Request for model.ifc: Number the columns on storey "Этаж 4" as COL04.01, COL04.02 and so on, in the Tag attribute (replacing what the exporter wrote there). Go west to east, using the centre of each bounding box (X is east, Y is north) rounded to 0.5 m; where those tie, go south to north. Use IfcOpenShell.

First a look at what the model holds.

```python
import ifcopenshell
import ifcopenshell.util.element
import ifcopenshell.util.placement

model = ifcopenshell.open("model.ifc")
print(model.schema)
storey = next(s for s in model.by_type("IfcBuildingStorey") if s.Name == "Этаж 4")
columns = [e for e in ifcopenshell.util.element.get_decomposition(storey) if e.is_a("IfcColumn")]
for e in sorted(columns, key=lambda e: e.id()):
    origin = ifcopenshell.util.placement.get_local_placement(e.ObjectPlacement)[:3, 3]
    print(e.id(), e.Tag, e.Name, origin.round(2) + 0.0, sep=" | ")
```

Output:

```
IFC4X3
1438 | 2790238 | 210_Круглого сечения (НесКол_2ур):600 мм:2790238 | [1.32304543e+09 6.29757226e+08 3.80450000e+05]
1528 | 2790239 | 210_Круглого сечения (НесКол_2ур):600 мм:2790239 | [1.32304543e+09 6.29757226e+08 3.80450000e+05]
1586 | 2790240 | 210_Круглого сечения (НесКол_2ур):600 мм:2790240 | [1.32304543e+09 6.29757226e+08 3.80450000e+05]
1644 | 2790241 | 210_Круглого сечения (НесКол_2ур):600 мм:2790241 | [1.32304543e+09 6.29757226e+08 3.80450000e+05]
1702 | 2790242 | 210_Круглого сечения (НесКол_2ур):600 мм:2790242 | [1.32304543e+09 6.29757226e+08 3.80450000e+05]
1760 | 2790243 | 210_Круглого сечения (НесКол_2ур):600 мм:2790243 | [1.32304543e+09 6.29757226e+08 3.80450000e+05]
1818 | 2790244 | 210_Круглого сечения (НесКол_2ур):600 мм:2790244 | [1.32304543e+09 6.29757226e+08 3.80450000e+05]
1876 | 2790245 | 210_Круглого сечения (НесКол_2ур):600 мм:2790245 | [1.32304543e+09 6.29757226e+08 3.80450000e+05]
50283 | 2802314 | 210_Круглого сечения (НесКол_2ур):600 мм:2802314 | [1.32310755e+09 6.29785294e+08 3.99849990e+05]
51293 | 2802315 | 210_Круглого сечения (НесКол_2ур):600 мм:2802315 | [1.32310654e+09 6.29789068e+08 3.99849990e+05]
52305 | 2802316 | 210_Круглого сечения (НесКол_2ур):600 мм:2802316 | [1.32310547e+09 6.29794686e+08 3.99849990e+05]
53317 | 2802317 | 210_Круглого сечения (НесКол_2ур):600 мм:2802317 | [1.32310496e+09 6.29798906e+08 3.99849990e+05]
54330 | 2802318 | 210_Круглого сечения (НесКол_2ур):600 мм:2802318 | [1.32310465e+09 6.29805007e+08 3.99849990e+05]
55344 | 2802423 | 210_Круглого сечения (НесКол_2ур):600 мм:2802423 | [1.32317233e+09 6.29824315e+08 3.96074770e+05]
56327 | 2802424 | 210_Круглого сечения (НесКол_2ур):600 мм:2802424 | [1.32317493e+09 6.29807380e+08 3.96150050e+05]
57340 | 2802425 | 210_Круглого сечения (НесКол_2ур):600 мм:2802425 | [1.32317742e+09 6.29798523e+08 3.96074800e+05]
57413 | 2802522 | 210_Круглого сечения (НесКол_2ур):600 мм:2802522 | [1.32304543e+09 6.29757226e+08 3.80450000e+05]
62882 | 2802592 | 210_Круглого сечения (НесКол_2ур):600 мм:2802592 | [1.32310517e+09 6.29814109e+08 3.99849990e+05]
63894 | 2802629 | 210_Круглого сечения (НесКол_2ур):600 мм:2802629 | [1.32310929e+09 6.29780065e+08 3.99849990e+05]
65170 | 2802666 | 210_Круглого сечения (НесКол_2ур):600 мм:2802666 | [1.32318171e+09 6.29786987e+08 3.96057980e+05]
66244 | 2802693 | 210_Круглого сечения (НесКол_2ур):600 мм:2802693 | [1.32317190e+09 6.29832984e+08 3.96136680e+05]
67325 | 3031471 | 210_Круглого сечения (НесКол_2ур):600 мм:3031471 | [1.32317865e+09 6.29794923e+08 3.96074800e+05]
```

```python
import ifcopenshell
import ifcopenshell.geom
import ifcopenshell.util.element
import ifcopenshell.util.shape

model = ifcopenshell.open("model.ifc")
settings = ifcopenshell.geom.settings()
settings.set("use-world-coords", True)


def centre(element):
    shape = ifcopenshell.geom.create_shape(settings, element)
    return ifcopenshell.util.shape.get_bbox_centroid(shape.geometry)


storey = next(s for s in model.by_type("IfcBuildingStorey") if s.Name == "Этаж 4")
columns = [e for e in ifcopenshell.util.element.get_decomposition(storey) if e.is_a("IfcColumn")]

# Insertion points can sit at a corner or the storey origin, so sort by the geometry (in metres).
centres = {e: centre(e) for e in columns}
columns.sort(key=lambda e: (round(centres[e][0] / 0.5), centres[e][1]))

for i, e in enumerate(columns, start=1):
    number = f"COL04.{i:02d}"
    e.Tag = number
    print(e.id(), number)

model.write("model_edited.ifc")
```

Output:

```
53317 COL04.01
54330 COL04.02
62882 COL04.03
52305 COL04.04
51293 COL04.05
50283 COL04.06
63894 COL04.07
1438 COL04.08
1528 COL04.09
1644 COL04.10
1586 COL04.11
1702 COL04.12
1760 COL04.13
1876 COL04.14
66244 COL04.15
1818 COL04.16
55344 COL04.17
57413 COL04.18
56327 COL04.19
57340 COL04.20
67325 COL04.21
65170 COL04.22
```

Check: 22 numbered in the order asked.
